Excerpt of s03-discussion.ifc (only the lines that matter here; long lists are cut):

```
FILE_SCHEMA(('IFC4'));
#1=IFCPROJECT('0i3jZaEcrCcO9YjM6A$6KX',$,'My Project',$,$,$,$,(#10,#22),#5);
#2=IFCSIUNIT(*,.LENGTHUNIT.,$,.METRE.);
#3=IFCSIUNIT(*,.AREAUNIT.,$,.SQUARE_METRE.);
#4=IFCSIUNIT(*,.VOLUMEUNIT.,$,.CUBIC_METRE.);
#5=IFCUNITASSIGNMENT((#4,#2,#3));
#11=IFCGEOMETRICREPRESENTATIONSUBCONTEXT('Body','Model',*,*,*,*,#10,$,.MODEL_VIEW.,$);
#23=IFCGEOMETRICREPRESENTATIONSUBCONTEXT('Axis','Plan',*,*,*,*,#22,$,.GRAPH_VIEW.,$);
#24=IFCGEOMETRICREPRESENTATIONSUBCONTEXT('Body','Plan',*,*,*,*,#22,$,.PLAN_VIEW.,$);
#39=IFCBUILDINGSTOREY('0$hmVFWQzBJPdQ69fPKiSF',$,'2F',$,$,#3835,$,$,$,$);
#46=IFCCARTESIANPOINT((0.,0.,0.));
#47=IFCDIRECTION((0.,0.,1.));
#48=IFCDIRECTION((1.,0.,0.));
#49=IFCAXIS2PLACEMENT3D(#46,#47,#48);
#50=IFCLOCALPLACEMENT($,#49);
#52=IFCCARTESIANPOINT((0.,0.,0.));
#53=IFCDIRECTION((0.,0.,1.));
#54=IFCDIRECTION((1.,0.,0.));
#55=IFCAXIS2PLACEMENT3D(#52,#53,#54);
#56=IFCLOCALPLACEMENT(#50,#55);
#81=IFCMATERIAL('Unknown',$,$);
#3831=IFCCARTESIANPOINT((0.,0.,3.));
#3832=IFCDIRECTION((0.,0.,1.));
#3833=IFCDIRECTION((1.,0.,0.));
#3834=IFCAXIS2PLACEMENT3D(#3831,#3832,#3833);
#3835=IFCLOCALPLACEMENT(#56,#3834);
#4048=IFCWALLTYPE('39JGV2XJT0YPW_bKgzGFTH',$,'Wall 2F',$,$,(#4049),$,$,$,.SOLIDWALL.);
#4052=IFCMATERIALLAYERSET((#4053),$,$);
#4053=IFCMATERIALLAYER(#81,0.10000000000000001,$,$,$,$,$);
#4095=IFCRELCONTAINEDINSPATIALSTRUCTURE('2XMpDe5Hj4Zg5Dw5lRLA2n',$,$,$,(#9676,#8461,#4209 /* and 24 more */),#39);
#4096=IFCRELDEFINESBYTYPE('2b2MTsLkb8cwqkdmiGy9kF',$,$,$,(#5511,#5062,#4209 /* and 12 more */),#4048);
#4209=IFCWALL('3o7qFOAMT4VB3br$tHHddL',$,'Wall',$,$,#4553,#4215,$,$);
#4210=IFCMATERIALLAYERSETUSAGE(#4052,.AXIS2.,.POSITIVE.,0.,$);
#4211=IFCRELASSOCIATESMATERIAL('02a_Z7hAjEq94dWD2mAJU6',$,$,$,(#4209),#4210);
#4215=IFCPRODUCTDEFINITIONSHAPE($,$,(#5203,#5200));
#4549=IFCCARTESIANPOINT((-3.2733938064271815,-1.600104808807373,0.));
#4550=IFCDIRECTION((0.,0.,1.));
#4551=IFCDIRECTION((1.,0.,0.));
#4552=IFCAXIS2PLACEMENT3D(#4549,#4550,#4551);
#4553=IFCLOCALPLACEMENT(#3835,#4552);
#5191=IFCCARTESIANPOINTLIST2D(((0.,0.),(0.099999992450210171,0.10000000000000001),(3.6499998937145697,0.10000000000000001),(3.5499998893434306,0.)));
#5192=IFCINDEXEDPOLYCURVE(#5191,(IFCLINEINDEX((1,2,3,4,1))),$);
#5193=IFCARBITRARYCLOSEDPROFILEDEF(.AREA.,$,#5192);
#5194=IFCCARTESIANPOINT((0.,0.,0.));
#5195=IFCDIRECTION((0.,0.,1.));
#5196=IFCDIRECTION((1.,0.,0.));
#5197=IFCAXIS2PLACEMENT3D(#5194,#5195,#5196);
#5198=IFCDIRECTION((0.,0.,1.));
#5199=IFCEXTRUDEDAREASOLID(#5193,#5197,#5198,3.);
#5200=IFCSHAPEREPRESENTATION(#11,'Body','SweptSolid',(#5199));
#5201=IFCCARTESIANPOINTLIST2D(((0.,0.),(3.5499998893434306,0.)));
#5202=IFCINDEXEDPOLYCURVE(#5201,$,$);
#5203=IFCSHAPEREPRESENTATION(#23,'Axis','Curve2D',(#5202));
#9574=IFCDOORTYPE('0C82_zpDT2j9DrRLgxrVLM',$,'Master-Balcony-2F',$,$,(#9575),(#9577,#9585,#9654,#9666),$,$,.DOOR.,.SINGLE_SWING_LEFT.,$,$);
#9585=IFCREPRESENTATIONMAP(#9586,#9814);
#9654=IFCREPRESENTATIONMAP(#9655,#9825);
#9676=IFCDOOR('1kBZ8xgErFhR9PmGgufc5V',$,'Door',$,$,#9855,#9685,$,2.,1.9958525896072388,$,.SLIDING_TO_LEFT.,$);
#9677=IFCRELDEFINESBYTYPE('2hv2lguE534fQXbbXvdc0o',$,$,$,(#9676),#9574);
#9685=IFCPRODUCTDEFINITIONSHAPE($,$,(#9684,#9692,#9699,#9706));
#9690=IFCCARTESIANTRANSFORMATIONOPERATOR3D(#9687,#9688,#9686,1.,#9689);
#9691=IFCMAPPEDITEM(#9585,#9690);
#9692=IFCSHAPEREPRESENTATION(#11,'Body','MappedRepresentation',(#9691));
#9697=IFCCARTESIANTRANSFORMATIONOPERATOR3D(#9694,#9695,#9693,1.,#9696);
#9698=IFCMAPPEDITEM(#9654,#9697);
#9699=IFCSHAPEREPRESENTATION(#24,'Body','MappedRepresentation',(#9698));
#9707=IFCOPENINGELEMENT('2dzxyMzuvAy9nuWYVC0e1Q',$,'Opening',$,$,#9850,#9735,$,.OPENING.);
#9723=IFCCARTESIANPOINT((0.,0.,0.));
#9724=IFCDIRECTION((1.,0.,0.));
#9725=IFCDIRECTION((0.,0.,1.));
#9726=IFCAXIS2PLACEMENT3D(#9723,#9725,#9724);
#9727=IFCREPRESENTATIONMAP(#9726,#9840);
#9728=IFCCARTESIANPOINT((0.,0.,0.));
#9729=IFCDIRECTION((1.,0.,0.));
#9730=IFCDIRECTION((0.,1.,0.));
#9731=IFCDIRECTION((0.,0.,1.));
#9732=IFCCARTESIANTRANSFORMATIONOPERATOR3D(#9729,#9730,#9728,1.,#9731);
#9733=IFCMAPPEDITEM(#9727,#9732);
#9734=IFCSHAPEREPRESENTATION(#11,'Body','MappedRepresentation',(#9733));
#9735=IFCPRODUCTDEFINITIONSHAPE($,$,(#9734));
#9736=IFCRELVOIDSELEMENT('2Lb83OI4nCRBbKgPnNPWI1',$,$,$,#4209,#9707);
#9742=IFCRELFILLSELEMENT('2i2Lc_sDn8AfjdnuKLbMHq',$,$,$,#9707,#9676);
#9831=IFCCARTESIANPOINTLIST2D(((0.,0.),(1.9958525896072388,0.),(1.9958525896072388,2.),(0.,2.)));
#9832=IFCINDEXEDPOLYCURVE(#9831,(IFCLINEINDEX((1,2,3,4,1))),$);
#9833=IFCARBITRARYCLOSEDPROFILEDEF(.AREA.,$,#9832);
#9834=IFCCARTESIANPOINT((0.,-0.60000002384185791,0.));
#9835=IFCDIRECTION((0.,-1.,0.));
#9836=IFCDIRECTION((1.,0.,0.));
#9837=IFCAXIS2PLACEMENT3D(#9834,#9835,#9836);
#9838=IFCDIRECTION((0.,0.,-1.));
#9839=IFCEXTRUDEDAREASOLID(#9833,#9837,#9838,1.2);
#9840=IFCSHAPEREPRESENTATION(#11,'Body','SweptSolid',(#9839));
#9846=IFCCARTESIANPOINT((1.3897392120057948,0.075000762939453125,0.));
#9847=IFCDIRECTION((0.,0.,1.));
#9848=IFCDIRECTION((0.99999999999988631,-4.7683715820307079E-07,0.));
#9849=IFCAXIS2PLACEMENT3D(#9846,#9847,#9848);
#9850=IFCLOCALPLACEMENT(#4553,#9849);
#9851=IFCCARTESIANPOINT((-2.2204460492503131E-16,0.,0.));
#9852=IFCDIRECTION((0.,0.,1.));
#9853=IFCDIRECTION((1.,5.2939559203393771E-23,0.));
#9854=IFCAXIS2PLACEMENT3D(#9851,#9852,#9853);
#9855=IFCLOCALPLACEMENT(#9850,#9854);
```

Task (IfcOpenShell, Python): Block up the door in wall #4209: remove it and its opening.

```python
import ifcopenshell
import ifcopenshell.api.feature
import ifcopenshell.api.root
import ifcopenshell.geom
import ifcopenshell.util.shape

model = ifcopenshell.open("s03-discussion.ifc")
settings = ifcopenshell.geom.settings()


def volume(element):
    """Net volume in cubic metres, openings subtracted."""
    shape = ifcopenshell.geom.create_shape(settings, element)
    return ifcopenshell.util.shape.get_volume(shape.geometry)


door = model.by_id(9676)
opening = door.FillsVoids[0].RelatingOpeningElement
wall = opening.VoidsElements[0].RelatingBuildingElement
before = volume(wall)

ifcopenshell.api.root.remove_product(model, product=door)
ifcopenshell.api.feature.remove_feature(model, feature=opening)

after = volume(wall)

print(f"wall volume {before:.3f} -> {after:.3f} m3")

model.write("s03-discussion-out.ifc")
```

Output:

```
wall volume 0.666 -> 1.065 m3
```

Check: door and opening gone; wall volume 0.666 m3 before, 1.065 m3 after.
